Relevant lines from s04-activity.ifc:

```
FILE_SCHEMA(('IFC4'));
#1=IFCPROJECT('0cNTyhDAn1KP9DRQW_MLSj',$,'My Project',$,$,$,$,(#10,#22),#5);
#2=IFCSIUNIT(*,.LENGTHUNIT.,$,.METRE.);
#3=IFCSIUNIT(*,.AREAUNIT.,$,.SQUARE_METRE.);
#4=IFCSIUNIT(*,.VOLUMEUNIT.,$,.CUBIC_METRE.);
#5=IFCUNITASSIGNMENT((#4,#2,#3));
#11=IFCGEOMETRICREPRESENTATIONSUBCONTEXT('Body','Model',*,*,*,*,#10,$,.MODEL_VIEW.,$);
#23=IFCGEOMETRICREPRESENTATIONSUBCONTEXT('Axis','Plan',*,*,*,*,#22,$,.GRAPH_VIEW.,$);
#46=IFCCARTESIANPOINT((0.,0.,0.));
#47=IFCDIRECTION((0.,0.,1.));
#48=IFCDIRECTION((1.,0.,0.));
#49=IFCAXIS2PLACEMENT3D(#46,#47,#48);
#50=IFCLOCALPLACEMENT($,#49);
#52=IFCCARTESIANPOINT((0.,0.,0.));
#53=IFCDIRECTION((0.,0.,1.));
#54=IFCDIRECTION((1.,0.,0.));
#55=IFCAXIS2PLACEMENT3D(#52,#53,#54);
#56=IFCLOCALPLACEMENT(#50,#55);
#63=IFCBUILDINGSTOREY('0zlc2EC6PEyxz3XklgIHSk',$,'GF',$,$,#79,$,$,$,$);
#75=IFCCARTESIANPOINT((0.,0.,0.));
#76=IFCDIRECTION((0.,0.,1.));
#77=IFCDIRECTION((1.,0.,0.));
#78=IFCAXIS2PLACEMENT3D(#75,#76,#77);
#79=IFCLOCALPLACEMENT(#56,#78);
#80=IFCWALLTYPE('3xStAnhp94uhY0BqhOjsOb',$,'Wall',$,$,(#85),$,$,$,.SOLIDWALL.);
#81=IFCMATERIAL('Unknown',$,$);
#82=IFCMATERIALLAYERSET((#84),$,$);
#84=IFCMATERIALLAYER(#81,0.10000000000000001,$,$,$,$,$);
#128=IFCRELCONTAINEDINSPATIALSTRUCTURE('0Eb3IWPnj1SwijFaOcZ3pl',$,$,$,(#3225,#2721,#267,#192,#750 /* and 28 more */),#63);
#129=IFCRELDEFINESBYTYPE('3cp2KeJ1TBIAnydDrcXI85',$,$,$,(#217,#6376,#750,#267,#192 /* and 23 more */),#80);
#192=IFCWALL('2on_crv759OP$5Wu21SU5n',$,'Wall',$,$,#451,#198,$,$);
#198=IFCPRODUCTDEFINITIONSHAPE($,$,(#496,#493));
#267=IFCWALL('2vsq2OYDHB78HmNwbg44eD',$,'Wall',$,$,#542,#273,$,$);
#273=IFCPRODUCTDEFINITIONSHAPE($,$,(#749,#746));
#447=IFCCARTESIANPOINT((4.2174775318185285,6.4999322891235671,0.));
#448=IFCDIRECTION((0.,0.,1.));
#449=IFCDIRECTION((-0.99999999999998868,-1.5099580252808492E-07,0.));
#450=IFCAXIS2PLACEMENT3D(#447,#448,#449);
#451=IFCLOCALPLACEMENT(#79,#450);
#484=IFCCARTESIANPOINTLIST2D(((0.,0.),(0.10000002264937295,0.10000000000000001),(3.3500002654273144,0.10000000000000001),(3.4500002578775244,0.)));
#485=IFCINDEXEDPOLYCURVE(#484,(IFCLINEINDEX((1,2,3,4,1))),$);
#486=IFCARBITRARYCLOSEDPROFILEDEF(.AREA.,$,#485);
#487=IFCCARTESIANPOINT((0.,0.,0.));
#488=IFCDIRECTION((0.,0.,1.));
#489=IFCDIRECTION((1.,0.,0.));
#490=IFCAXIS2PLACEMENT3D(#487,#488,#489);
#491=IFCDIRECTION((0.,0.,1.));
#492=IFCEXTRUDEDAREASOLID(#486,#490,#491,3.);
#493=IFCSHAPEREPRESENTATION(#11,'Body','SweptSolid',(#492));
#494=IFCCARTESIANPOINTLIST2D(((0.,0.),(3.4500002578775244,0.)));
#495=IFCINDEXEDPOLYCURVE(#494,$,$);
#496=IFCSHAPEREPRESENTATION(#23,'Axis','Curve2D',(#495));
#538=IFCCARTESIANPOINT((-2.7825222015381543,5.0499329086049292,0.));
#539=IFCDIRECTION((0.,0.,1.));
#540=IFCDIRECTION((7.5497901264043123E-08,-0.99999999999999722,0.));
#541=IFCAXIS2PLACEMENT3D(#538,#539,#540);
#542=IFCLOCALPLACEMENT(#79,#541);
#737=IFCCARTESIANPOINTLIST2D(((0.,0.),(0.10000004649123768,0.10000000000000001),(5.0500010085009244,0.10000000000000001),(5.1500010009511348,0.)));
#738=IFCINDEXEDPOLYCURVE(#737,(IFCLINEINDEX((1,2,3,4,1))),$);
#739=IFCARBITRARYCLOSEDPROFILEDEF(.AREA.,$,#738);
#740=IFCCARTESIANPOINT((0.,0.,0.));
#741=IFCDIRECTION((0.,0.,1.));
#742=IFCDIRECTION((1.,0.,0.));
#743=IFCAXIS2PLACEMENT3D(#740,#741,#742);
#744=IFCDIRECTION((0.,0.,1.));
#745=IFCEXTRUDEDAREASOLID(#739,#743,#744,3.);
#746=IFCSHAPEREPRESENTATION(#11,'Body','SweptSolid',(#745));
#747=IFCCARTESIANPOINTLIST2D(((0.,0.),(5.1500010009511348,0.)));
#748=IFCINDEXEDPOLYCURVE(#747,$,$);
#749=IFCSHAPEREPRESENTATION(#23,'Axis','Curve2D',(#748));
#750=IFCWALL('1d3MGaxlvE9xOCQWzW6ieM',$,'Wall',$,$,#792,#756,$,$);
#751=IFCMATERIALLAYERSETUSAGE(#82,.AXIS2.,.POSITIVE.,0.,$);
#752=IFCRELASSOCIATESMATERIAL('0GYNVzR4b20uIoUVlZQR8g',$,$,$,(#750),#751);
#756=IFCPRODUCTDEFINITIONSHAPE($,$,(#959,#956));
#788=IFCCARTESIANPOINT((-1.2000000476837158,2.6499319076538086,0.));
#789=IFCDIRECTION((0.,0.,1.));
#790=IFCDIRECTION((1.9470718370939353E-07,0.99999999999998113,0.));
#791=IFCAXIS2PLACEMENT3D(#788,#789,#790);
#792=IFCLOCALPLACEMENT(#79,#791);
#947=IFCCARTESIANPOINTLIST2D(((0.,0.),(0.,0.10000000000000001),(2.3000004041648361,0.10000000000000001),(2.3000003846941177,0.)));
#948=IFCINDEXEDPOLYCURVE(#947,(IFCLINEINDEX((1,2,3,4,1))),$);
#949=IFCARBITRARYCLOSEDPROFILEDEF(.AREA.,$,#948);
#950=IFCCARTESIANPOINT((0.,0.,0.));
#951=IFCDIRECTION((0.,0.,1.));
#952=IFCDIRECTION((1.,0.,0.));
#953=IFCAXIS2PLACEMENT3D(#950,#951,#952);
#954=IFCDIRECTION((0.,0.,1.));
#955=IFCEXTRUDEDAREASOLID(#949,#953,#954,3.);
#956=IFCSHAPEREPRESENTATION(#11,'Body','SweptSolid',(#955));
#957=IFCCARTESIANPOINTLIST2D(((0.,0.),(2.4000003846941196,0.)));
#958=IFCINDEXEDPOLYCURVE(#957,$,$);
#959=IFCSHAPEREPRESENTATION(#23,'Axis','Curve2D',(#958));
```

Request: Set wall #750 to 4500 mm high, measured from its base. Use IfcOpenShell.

```python
import ifcopenshell
import ifcopenshell.geom
import ifcopenshell.util.representation
import ifcopenshell.util.shape
import ifcopenshell.util.unit

model = ifcopenshell.open("s04-activity.ifc")
unit_scale = ifcopenshell.util.unit.calculate_unit_scale(model)
settings = ifcopenshell.geom.settings()


def volume(element):
    """Net volume in cubic metres, openings subtracted."""
    shape = ifcopenshell.geom.create_shape(settings, element)
    return ifcopenshell.util.shape.get_volume(shape.geometry)


wall = model.by_guid("1d3MGaxlvE9xOCQWzW6ieM")
before = volume(wall)

body = ifcopenshell.util.representation.get_representation(wall, "Model", "Body")
solid = body.Items[0]
old_height = solid.Depth
solid.Depth = 4.5 / unit_scale
after = volume(wall)

print(f"height {old_height:g} -> {solid.Depth:g}, volume {before:.3f} -> {after:.3f} m3")

model.write("s04-activity-out.ifc")
```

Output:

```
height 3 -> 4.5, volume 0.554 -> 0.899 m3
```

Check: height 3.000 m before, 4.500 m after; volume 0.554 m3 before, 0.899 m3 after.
